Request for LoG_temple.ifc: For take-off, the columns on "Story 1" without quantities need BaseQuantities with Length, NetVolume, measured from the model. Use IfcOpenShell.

First a look at what the model holds.

```python
import ifcopenshell
import ifcopenshell.util.element
import ifcopenshell.util.unit

model = ifcopenshell.open("LoG_temple.ifc")
print(model.schema)
for unit_type in ("LENGTHUNIT", "AREAUNIT", "VOLUMEUNIT"):
    print(unit_type, ifcopenshell.util.unit.calculate_unit_scale(model, unit_type))
storey = next(s for s in model.by_type("IfcBuildingStorey") if s.Name == "Story 1")
columns = [e for e in ifcopenshell.util.element.get_decomposition(storey) if e.is_a("IfcColumn")]
for e in sorted(columns, key=lambda e: e.id()):
    print(e.id(), e.is_a(), e.Name, list(ifcopenshell.util.element.get_psets(e, qtos_only=True)), sep=" | ")
```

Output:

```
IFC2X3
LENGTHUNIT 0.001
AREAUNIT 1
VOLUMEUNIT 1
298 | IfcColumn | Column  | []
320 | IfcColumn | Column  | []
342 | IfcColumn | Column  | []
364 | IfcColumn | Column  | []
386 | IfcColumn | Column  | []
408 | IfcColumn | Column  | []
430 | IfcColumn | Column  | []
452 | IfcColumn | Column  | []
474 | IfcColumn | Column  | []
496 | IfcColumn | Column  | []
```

```python
import ifcopenshell
import ifcopenshell.api.pset
import ifcopenshell.geom
import ifcopenshell.util.element
import ifcopenshell.util.shape
import ifcopenshell.util.unit

model = ifcopenshell.open("LoG_temple.ifc")
unit_scale = ifcopenshell.util.unit.calculate_unit_scale(model)
volume_scale = ifcopenshell.util.unit.calculate_unit_scale(model, "VOLUMEUNIT")
settings = ifcopenshell.geom.settings()

storey = next(s for s in model.by_type("IfcBuildingStorey") if s.Name == "Story 1")
columns = [e for e in ifcopenshell.util.element.get_decomposition(storey) if e.is_a("IfcColumn")]

for e in sorted(columns, key=lambda e: e.id()):
    if ifcopenshell.util.element.get_psets(e, qtos_only=True, should_inherit=False):
        continue
    # Geometry comes back in metres, in the element's own axes.
    shape = ifcopenshell.geom.create_shape(settings, e)
    values = {
        "Length": ifcopenshell.util.shape.get_z(shape.geometry) / unit_scale,
        "NetVolume": ifcopenshell.util.shape.get_volume(shape.geometry) / volume_scale,
    }
    qto = ifcopenshell.api.pset.add_qto(model, product=e, name="BaseQuantities")
    ifcopenshell.api.pset.edit_qto(model, qto=qto, properties=values)
    print(e.id(), {k: round(v, 3) for k, v in values.items()})

model.write("LoG_temple_rev.ifc")
```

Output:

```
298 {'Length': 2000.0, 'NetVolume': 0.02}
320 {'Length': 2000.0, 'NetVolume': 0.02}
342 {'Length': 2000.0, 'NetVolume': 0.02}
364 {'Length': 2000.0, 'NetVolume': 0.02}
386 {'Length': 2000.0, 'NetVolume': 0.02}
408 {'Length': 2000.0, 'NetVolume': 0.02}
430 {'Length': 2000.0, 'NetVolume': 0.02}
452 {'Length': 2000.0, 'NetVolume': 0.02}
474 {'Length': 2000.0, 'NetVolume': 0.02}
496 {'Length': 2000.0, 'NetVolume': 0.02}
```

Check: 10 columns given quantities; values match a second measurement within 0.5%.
